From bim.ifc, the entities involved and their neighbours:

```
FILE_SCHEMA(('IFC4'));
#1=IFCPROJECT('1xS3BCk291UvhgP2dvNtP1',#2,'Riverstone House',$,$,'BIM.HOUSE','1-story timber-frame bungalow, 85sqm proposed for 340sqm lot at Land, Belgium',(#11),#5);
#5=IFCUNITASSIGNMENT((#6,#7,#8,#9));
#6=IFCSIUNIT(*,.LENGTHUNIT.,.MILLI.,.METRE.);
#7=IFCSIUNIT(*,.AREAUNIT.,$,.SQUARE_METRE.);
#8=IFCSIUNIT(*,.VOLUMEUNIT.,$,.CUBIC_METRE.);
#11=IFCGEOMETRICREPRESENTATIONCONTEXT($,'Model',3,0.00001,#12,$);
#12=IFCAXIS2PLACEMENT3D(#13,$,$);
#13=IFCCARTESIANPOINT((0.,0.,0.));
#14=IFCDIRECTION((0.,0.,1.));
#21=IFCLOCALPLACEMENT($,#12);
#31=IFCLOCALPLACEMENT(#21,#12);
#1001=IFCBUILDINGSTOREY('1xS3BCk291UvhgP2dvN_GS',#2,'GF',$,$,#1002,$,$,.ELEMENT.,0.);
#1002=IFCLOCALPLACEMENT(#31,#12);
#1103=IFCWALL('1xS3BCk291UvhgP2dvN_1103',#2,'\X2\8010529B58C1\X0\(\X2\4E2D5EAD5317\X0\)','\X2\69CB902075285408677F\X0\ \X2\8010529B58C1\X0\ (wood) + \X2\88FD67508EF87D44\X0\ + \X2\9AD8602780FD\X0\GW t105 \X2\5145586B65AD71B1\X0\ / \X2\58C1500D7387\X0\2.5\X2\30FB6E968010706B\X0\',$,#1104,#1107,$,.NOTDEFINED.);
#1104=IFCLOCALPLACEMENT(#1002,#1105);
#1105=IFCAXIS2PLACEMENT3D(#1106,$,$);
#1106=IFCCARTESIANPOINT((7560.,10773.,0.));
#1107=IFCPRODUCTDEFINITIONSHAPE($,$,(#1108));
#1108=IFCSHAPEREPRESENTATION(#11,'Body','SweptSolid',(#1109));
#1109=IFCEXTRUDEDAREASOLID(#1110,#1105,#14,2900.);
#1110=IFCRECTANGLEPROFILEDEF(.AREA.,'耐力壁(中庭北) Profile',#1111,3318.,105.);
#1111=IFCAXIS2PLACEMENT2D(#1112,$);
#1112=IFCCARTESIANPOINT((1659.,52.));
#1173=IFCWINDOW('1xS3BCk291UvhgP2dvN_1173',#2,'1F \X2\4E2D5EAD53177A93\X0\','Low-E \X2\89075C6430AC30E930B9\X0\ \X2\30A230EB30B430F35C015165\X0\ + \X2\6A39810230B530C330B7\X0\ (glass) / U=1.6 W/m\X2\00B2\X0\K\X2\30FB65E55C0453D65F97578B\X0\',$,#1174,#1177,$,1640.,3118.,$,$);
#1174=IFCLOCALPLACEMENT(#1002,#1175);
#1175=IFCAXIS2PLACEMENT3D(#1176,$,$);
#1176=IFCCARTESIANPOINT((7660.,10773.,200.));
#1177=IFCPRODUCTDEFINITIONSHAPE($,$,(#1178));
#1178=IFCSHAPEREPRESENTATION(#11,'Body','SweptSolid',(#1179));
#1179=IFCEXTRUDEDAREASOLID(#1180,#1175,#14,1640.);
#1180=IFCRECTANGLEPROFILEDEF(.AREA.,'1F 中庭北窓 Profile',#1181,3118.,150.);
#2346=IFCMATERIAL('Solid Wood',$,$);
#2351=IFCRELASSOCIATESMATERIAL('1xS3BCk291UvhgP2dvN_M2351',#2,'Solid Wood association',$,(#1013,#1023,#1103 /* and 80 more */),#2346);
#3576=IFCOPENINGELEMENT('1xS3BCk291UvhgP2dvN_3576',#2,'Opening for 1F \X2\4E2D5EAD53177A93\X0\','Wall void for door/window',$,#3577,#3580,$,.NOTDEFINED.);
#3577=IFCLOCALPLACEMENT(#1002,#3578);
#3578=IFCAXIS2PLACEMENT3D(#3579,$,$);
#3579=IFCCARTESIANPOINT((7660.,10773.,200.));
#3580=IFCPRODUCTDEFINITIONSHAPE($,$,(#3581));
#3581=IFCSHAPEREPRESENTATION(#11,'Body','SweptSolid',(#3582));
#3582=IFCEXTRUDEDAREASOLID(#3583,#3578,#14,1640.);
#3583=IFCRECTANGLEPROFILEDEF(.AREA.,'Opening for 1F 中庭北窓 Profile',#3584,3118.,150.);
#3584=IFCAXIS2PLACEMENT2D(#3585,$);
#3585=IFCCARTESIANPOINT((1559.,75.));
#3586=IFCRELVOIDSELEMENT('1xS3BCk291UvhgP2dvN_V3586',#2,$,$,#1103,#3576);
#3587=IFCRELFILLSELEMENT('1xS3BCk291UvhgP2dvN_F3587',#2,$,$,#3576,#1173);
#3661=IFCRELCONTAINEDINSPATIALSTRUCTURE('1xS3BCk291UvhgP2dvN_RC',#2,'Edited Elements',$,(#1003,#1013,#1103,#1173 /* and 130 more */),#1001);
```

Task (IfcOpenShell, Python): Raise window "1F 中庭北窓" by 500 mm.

```python
import numpy as np
import ifcopenshell
import ifcopenshell.api.geometry
import ifcopenshell.util.placement
import ifcopenshell.util.unit

model = ifcopenshell.open("bim.ifc")
unit_scale = ifcopenshell.util.unit.calculate_unit_scale(model)

window = model.by_guid("1xS3BCk291UvhgP2dvN_1173")
opening = window.FillsVoids[0].RelatingOpeningElement
dz = 0.5 / unit_scale

shift = np.array([0.0, 0.0, dz])
# The window is not placed relative to its opening, so move both.
for product in (opening, window):
    matrix = ifcopenshell.util.placement.get_local_placement(product.ObjectPlacement)
    matrix[:3, 3] += shift
    ifcopenshell.api.geometry.edit_object_placement(model, product=product, matrix=matrix, is_si=False)

print(f"moved by {dz * unit_scale:+.3f} m")

model.write("bim_edited.ifc")
```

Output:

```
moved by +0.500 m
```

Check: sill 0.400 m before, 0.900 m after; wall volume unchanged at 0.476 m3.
